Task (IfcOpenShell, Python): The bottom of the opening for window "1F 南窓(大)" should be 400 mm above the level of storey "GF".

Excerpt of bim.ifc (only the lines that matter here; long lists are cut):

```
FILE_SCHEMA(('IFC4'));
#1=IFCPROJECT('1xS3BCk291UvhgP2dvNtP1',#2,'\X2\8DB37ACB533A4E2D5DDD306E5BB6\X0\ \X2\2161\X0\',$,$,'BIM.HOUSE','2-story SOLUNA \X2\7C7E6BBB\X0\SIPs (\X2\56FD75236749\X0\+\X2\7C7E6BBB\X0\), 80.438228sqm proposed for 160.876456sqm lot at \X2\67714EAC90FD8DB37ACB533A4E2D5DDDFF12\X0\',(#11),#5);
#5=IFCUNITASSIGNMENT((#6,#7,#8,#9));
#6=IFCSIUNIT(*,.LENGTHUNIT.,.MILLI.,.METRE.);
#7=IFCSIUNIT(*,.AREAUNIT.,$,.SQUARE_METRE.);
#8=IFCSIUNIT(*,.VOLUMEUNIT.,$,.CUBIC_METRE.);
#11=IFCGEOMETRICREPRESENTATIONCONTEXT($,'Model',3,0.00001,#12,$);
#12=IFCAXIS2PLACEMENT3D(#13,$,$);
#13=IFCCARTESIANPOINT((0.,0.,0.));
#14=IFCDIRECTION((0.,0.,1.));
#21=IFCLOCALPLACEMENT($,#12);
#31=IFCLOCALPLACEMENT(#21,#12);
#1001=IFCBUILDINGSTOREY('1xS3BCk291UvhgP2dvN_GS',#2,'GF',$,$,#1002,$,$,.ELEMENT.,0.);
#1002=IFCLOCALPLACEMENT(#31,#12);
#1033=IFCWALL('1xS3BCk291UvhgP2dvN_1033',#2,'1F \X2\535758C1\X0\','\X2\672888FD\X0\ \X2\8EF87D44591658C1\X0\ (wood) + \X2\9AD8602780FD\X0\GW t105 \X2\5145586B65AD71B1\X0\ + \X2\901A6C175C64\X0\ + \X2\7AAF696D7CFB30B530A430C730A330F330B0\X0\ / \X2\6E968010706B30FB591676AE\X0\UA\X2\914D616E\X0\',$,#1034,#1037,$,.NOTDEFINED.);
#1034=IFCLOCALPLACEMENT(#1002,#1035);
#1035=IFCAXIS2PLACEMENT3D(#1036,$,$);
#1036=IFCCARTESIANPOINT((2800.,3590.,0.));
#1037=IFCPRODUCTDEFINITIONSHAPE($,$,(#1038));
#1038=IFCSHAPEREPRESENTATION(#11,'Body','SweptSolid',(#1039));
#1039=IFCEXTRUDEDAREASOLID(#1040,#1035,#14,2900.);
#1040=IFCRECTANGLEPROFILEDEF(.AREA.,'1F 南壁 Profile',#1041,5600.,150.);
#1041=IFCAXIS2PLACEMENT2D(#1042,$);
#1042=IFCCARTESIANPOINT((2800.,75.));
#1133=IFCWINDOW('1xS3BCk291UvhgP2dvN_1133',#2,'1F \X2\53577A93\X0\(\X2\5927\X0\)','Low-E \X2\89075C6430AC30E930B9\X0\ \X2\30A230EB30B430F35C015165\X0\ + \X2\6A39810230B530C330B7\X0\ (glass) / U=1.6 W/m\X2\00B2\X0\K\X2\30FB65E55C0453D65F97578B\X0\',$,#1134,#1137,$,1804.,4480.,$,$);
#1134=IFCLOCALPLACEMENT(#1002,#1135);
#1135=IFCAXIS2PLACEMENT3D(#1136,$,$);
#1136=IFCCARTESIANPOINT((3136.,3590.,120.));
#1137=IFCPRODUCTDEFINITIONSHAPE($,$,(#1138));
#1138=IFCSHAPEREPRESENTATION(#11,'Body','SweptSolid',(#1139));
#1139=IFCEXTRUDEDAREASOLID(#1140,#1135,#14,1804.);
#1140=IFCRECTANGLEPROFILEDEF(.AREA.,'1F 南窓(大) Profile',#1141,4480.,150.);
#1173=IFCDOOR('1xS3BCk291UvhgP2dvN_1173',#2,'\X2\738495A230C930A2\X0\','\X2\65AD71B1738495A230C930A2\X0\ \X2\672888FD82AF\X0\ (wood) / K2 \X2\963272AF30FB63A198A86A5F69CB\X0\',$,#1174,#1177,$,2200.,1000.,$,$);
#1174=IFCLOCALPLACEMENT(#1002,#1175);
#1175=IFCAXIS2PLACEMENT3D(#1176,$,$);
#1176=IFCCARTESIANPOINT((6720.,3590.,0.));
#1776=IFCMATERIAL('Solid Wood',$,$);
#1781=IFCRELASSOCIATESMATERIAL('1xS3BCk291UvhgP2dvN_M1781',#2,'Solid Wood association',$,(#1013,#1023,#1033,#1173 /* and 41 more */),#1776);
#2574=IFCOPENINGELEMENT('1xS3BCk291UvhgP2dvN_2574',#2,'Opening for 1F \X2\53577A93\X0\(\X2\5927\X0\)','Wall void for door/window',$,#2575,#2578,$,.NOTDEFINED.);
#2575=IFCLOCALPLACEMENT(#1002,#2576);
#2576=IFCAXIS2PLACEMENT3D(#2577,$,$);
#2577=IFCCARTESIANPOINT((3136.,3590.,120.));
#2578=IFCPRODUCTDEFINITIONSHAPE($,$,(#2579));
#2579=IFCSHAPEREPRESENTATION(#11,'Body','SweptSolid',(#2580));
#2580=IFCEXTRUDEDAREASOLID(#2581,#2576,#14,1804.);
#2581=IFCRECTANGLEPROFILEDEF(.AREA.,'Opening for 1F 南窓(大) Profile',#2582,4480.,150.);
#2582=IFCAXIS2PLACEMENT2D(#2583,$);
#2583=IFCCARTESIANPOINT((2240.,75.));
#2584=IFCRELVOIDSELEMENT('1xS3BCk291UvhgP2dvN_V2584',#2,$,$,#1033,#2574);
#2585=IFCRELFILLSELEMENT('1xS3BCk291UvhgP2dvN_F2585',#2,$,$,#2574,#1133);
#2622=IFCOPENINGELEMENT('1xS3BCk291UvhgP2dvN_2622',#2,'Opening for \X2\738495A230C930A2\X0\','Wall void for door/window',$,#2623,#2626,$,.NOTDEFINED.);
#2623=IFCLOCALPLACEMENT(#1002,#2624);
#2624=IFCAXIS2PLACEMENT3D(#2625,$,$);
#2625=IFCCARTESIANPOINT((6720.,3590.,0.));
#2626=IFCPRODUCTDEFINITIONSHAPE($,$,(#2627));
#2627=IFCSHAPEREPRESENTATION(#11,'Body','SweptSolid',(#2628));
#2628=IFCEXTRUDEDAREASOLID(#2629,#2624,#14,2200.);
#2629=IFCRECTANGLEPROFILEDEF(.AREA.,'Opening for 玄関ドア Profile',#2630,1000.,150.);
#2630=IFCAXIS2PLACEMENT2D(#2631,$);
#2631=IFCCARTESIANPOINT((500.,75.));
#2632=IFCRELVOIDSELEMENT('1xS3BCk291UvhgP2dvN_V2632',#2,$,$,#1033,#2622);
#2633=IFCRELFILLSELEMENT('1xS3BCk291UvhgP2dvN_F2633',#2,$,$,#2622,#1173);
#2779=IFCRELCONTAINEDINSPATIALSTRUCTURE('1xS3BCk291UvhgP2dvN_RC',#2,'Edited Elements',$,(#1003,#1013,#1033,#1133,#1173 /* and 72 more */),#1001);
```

```python
import numpy as np
import ifcopenshell
import ifcopenshell.api.geometry
import ifcopenshell.geom
import ifcopenshell.util.element
import ifcopenshell.util.placement
import ifcopenshell.util.shape
import ifcopenshell.util.unit

model = ifcopenshell.open("bim.ifc")
unit_scale = ifcopenshell.util.unit.calculate_unit_scale(model)

window = model.by_guid("1xS3BCk291UvhgP2dvN_1133")
opening = window.FillsVoids[0].RelatingOpeningElement
storey = ifcopenshell.util.element.get_container(window, ifc_class="IfcBuildingStorey")
level = ifcopenshell.util.placement.get_local_placement(storey.ObjectPlacement)[2, 3]

# The opening's origin need not be at the sill, so measure its lowest point.
shape = ifcopenshell.geom.create_shape(ifcopenshell.geom.settings(), opening)
bottom = ifcopenshell.util.shape.get_shape_bottom_elevation(shape, shape.geometry) / unit_scale
dz = level + 400.0 - bottom

shift = np.array([0.0, 0.0, dz])
# The window is not placed relative to its opening, so move both.
for product in (opening, window):
    matrix = ifcopenshell.util.placement.get_local_placement(product.ObjectPlacement)
    matrix[:3, 3] += shift
    ifcopenshell.api.geometry.edit_object_placement(model, product=product, matrix=matrix, is_si=False)

print(f"moved by {dz * unit_scale:+.3f} m")

model.write("bim_v2.ifc")
```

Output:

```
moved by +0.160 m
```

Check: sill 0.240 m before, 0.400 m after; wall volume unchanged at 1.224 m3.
